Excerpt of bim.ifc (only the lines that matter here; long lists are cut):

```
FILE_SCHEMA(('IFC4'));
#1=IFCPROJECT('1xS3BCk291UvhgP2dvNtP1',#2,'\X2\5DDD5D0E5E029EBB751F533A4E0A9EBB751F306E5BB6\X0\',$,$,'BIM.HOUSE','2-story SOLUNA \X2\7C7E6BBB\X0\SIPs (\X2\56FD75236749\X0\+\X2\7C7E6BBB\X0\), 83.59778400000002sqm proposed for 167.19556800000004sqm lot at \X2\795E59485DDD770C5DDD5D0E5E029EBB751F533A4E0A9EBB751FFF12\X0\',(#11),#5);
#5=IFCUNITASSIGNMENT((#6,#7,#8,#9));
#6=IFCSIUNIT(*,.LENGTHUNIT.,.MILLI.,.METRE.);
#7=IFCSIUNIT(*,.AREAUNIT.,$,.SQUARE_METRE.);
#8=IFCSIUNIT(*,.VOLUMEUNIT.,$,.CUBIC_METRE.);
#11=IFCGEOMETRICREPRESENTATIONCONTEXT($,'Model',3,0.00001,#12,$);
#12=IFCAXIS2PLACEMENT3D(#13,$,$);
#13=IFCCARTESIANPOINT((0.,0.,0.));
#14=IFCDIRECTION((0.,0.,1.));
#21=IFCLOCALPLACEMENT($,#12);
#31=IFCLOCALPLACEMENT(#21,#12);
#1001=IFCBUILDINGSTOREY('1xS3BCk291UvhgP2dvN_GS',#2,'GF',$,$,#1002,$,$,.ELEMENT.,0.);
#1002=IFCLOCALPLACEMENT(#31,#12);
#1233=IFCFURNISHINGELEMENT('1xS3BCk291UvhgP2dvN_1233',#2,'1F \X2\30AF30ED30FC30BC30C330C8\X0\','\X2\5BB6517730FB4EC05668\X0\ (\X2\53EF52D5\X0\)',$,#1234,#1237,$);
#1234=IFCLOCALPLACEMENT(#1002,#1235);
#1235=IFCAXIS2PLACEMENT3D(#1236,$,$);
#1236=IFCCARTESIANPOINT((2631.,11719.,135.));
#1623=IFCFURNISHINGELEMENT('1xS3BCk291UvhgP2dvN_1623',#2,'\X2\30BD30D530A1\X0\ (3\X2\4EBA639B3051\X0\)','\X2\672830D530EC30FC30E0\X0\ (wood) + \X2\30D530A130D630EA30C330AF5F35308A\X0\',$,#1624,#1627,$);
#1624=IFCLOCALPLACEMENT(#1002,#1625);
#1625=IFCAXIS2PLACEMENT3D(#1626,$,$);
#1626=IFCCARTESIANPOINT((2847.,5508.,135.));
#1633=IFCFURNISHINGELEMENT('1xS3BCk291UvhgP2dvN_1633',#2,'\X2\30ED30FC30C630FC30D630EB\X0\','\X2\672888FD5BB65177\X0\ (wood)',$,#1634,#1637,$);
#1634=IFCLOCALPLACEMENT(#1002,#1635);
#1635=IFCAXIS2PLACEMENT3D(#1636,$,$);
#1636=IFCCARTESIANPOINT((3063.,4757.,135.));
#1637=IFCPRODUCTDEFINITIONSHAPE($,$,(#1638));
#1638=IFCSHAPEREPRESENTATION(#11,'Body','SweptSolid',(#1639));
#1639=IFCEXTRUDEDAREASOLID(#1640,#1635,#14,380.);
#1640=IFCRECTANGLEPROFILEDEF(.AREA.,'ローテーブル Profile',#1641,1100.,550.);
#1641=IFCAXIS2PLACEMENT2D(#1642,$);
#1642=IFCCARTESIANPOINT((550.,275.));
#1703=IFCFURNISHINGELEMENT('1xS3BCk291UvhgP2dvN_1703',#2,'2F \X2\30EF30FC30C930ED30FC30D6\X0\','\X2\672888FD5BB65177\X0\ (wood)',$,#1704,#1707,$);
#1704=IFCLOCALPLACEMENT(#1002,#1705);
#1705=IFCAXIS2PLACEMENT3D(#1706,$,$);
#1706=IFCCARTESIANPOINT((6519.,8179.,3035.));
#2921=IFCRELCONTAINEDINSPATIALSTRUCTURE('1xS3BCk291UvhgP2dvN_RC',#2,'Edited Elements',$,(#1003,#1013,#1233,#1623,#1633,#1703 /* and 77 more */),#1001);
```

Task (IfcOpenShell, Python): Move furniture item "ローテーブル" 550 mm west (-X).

```python
import ifcopenshell
import ifcopenshell.api.geometry
import ifcopenshell.util.placement
import ifcopenshell.util.unit

model = ifcopenshell.open("bim.ifc")
unit_scale = ifcopenshell.util.unit.calculate_unit_scale(model)

item = model.by_guid("1xS3BCk291UvhgP2dvN_1633")
matrix = ifcopenshell.util.placement.get_local_placement(item.ObjectPlacement)
matrix[0, 3] -= 0.55 / unit_scale
ifcopenshell.api.geometry.edit_object_placement(model, product=item, matrix=matrix, is_si=False)

print(ifcopenshell.util.placement.get_local_placement(item.ObjectPlacement).round(3) + 0.0)

model.write("bim-out.ifc")
```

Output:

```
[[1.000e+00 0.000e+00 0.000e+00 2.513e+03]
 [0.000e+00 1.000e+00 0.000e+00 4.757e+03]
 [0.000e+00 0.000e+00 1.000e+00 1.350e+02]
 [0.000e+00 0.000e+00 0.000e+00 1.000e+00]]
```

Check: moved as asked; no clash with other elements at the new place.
